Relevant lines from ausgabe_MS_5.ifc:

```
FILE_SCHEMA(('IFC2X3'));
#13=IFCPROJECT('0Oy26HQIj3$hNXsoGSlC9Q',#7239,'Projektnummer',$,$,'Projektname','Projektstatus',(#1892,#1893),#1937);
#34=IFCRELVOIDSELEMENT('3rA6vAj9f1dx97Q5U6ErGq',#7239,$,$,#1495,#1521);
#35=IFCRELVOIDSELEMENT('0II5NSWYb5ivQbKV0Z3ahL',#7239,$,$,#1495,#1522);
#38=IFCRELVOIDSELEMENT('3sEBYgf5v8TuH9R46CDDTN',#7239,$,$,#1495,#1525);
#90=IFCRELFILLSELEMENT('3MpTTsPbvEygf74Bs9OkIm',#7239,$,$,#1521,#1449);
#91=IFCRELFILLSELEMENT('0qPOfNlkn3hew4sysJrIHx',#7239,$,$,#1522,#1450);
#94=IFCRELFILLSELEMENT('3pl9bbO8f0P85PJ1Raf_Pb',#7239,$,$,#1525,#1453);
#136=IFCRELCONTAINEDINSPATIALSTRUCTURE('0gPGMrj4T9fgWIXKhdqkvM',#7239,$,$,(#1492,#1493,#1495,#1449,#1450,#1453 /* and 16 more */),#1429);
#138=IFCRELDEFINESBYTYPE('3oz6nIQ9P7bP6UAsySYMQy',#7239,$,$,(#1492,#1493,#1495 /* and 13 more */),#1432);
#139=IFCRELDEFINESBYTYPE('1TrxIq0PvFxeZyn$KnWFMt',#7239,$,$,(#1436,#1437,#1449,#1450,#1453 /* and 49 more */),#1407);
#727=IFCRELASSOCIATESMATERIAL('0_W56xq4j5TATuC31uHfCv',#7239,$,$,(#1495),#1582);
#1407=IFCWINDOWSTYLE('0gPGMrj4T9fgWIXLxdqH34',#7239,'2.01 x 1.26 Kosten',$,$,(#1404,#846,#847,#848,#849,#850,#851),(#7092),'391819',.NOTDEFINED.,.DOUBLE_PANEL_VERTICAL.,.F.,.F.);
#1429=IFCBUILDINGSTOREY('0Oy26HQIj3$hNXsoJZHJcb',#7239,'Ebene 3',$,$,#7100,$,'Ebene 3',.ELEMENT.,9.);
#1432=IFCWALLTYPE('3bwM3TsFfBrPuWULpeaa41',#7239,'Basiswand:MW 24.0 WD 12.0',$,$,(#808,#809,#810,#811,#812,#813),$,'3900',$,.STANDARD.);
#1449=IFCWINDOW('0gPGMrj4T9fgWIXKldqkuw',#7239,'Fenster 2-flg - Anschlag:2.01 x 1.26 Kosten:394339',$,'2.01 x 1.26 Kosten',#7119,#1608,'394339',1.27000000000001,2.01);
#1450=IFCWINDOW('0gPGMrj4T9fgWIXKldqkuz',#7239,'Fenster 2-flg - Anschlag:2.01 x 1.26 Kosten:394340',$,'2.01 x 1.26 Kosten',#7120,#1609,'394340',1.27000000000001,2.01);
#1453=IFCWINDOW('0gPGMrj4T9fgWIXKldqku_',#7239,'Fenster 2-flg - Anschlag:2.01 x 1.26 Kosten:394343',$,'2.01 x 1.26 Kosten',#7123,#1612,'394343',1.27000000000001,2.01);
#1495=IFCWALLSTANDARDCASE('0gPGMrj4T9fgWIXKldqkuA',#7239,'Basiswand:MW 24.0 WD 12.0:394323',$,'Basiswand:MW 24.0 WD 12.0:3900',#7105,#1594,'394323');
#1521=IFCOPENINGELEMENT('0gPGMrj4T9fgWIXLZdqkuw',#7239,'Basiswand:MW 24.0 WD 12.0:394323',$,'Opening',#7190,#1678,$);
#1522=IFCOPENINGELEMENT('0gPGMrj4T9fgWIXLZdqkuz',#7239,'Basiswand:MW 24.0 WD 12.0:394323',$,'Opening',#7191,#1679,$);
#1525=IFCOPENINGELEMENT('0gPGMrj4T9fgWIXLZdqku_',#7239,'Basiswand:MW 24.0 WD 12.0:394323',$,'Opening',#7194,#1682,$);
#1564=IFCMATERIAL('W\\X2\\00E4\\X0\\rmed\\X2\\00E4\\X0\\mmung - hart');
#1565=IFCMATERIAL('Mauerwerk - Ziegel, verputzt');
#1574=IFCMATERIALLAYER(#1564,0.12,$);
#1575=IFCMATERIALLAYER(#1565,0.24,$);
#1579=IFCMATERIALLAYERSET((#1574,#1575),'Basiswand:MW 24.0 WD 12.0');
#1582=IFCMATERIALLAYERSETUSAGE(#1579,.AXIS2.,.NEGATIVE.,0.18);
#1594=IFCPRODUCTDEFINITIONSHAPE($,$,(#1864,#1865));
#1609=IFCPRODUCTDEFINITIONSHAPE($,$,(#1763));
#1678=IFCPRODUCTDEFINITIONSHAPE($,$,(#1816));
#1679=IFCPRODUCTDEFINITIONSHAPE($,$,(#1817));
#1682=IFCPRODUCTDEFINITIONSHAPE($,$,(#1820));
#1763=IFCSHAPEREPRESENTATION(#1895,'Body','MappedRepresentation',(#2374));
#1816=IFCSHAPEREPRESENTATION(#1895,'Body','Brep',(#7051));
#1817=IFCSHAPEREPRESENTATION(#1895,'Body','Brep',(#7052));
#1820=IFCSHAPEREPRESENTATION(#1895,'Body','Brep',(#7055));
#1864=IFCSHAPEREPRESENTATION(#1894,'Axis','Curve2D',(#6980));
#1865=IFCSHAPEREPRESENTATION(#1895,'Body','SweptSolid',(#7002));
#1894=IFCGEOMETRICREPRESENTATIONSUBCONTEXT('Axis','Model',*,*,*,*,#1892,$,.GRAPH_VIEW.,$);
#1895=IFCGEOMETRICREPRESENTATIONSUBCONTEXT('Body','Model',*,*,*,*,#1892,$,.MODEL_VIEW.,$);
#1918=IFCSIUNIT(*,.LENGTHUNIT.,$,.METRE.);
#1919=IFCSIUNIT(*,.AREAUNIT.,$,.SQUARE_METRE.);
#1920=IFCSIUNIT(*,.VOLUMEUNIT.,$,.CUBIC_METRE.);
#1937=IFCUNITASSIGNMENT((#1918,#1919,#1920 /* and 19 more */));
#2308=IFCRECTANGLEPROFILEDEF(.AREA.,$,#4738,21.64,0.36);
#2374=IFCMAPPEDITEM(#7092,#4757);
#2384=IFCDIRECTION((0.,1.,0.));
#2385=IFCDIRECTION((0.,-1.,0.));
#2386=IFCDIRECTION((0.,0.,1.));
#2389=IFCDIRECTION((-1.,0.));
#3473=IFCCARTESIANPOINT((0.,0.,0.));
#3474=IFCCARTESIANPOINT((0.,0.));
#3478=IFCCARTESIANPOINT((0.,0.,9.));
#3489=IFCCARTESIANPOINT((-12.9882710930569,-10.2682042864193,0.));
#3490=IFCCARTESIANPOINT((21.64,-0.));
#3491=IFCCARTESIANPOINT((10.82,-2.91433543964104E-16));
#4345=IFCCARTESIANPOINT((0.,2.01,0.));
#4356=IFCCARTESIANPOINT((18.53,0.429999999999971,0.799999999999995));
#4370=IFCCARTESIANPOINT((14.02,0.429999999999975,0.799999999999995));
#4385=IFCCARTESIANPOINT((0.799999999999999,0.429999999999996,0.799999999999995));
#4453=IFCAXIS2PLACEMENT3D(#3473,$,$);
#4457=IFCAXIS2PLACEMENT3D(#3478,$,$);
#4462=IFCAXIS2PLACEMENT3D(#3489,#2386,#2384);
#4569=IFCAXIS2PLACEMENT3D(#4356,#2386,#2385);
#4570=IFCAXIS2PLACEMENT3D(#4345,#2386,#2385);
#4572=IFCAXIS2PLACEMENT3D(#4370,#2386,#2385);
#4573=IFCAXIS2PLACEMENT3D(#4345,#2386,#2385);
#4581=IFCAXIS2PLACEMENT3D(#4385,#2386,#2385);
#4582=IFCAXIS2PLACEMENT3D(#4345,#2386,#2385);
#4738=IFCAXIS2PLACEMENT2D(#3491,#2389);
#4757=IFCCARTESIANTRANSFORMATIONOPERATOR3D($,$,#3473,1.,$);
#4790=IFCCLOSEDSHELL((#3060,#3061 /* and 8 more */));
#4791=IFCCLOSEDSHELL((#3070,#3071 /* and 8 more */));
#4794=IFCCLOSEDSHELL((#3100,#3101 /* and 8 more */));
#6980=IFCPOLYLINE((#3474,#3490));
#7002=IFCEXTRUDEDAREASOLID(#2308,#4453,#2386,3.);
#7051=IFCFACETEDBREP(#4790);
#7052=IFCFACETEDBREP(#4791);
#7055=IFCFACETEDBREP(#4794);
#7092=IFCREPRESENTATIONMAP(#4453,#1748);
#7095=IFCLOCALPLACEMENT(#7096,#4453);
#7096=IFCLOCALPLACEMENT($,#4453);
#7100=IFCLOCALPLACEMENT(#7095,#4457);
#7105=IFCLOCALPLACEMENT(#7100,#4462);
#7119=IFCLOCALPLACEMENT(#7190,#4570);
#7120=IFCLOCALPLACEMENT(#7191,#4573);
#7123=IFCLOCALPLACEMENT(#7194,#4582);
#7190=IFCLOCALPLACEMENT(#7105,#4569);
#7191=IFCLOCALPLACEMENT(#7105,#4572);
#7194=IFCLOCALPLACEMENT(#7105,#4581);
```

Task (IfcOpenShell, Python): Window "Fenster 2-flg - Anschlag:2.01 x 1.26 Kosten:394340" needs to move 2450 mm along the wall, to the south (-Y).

```python
import ifcopenshell
import ifcopenshell.api.geometry
import ifcopenshell.util.placement
import ifcopenshell.util.unit

model = ifcopenshell.open("ausgabe_MS_5.ifc")
unit_scale = ifcopenshell.util.unit.calculate_unit_scale(model)

window = model.by_id(1450)
opening = window.FillsVoids[0].RelatingOpeningElement
wall = opening.VoidsElements[0].RelatingBuildingElement

wall_matrix = ifcopenshell.util.placement.get_local_placement(wall.ObjectPlacement)
shift = wall_matrix[:3, 0] * -2.45 / unit_scale
before = ifcopenshell.util.placement.get_local_placement(window.ObjectPlacement)[:3, 3].copy()

# The window is placed relative to its opening, so it follows when the opening moves.
matrix = ifcopenshell.util.placement.get_local_placement(opening.ObjectPlacement)
matrix[:3, 3] += shift
ifcopenshell.api.geometry.edit_object_placement(
    model, product=opening, matrix=matrix, is_si=False, should_transform_children=True
)

after = ifcopenshell.util.placement.get_local_placement(window.ObjectPlacement)[:3, 3]
print("window moved by", (after - before).round(3) + 0.0)

model.write("ausgabe_MS_5_rev.ifc")
```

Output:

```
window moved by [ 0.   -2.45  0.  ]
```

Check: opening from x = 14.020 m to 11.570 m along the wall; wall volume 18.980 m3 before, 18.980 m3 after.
